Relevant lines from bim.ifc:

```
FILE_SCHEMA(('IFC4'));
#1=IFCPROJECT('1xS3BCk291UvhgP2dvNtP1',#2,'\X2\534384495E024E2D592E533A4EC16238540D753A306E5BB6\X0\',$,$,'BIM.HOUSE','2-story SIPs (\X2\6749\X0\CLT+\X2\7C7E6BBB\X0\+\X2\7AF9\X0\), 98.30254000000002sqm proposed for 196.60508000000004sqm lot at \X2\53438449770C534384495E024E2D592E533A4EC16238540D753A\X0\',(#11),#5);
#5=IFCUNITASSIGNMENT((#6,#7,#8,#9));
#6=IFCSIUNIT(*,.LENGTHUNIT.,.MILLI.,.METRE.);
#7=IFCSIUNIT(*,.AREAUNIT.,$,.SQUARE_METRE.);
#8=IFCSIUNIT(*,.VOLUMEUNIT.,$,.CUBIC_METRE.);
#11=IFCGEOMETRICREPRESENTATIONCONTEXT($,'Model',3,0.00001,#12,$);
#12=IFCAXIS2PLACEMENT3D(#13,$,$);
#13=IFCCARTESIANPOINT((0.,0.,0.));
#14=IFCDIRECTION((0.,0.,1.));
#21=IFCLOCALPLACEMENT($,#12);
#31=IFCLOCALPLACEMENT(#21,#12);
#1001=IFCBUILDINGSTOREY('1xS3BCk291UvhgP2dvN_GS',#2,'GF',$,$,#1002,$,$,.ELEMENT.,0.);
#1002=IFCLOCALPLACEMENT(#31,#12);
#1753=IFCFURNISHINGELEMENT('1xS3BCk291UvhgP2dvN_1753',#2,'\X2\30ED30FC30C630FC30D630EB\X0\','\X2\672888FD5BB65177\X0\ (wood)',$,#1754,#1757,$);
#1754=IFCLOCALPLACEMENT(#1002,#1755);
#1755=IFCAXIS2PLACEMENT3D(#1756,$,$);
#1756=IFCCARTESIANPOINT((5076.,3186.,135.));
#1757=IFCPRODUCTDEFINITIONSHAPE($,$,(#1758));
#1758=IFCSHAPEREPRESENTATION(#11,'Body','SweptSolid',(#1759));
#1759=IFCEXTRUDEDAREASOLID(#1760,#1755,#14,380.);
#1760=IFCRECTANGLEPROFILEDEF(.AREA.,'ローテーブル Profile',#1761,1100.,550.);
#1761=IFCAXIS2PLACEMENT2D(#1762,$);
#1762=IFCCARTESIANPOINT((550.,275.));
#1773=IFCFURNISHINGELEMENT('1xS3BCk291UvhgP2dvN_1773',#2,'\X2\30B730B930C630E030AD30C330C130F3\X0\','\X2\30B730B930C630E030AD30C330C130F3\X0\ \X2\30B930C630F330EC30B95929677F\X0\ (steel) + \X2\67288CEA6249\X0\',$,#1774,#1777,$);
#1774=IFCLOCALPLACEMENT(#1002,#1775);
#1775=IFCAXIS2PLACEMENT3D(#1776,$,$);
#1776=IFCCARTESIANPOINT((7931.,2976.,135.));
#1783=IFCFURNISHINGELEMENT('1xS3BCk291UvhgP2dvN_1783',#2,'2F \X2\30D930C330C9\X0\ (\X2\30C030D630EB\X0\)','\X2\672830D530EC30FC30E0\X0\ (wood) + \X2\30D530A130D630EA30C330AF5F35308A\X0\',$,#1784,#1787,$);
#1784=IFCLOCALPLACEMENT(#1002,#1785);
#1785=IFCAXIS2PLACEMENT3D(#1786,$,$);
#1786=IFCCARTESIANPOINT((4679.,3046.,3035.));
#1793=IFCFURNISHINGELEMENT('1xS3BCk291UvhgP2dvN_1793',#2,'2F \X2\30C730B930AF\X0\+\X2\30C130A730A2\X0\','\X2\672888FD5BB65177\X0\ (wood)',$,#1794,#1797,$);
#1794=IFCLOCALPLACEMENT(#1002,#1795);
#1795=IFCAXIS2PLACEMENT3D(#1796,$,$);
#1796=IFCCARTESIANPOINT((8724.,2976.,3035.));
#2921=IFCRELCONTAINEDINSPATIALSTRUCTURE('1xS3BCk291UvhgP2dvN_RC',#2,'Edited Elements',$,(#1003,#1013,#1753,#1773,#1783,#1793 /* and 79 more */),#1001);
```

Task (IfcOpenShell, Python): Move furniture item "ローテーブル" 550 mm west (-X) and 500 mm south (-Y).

```python
import ifcopenshell
import ifcopenshell.api.geometry
import ifcopenshell.util.placement

model = ifcopenshell.open("bim.ifc")

item = model.by_id(1753)
matrix = ifcopenshell.util.placement.get_local_placement(item.ObjectPlacement)
matrix[0, 3] -= 550.0
matrix[1, 3] -= 500.0
ifcopenshell.api.geometry.edit_object_placement(model, product=item, matrix=matrix, is_si=False)

print(ifcopenshell.util.placement.get_local_placement(item.ObjectPlacement).round(3) + 0.0)

model.write("bim_edited.ifc")
```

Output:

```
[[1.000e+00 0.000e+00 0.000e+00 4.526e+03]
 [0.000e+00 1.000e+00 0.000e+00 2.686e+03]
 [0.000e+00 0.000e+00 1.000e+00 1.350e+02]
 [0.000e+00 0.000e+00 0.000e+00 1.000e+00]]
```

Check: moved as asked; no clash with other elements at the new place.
